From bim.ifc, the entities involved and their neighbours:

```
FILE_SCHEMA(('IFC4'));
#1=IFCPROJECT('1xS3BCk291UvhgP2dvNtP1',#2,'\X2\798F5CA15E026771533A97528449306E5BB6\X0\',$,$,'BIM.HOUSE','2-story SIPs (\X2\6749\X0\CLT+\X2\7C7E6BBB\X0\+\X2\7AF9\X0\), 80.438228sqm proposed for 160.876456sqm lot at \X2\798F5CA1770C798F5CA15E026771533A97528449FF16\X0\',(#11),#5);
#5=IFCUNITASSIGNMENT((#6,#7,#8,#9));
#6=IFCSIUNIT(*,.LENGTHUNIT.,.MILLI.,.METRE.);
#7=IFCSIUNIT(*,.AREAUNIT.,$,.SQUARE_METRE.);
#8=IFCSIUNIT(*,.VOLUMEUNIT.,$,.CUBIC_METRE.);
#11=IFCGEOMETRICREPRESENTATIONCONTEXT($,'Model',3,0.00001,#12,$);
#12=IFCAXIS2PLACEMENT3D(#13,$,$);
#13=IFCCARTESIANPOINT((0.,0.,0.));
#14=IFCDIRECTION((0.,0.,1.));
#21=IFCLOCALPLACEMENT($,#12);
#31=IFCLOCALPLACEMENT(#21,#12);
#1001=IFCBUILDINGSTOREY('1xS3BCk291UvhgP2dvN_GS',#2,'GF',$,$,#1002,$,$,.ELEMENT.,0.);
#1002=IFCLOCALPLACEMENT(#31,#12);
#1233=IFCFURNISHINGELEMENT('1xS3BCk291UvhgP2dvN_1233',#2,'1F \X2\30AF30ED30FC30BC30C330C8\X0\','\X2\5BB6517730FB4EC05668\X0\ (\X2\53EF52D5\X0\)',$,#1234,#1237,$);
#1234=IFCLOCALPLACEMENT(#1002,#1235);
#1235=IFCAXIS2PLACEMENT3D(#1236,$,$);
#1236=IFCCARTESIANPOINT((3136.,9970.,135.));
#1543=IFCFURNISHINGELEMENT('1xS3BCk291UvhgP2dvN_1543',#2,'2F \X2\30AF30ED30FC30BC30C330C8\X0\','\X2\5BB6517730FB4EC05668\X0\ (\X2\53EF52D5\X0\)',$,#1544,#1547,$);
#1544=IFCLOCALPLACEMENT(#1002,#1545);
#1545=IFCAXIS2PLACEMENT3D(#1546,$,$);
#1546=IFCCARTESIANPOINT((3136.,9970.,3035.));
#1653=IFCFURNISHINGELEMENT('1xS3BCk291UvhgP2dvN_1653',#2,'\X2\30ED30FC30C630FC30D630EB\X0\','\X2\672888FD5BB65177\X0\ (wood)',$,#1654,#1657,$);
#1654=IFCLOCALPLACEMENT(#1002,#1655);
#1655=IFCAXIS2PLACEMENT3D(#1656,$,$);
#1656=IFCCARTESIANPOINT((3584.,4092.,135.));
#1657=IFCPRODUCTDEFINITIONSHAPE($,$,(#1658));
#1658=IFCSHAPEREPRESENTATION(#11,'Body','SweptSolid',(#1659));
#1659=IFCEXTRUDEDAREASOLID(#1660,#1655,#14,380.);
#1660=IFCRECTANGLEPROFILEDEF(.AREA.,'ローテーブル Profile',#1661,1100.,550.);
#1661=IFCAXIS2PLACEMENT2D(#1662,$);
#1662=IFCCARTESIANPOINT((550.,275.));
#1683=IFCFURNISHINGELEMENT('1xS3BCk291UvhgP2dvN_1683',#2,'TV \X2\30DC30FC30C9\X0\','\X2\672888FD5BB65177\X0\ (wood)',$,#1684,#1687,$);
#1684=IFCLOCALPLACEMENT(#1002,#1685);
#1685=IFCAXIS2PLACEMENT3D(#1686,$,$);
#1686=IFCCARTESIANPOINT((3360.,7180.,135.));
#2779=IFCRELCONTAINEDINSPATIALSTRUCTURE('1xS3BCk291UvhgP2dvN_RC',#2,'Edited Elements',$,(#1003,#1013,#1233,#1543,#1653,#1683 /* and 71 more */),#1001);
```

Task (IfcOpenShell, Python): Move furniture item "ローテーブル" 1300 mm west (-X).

```python
import ifcopenshell
import ifcopenshell.api.geometry
import ifcopenshell.util.placement
import ifcopenshell.util.unit

model = ifcopenshell.open("bim.ifc")
unit_scale = ifcopenshell.util.unit.calculate_unit_scale(model)

item = model.by_guid("1xS3BCk291UvhgP2dvN_1653")
matrix = ifcopenshell.util.placement.get_local_placement(item.ObjectPlacement)
matrix[0, 3] -= 1.3 / unit_scale
ifcopenshell.api.geometry.edit_object_placement(model, product=item, matrix=matrix, is_si=False)

print(ifcopenshell.util.placement.get_local_placement(item.ObjectPlacement).round(3) + 0.0)

model.write("bim_v2.ifc")
```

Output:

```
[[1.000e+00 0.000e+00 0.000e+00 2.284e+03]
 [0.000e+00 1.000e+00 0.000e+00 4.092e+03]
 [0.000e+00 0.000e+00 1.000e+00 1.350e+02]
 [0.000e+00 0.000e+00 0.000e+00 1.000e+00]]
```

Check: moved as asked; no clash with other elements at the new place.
